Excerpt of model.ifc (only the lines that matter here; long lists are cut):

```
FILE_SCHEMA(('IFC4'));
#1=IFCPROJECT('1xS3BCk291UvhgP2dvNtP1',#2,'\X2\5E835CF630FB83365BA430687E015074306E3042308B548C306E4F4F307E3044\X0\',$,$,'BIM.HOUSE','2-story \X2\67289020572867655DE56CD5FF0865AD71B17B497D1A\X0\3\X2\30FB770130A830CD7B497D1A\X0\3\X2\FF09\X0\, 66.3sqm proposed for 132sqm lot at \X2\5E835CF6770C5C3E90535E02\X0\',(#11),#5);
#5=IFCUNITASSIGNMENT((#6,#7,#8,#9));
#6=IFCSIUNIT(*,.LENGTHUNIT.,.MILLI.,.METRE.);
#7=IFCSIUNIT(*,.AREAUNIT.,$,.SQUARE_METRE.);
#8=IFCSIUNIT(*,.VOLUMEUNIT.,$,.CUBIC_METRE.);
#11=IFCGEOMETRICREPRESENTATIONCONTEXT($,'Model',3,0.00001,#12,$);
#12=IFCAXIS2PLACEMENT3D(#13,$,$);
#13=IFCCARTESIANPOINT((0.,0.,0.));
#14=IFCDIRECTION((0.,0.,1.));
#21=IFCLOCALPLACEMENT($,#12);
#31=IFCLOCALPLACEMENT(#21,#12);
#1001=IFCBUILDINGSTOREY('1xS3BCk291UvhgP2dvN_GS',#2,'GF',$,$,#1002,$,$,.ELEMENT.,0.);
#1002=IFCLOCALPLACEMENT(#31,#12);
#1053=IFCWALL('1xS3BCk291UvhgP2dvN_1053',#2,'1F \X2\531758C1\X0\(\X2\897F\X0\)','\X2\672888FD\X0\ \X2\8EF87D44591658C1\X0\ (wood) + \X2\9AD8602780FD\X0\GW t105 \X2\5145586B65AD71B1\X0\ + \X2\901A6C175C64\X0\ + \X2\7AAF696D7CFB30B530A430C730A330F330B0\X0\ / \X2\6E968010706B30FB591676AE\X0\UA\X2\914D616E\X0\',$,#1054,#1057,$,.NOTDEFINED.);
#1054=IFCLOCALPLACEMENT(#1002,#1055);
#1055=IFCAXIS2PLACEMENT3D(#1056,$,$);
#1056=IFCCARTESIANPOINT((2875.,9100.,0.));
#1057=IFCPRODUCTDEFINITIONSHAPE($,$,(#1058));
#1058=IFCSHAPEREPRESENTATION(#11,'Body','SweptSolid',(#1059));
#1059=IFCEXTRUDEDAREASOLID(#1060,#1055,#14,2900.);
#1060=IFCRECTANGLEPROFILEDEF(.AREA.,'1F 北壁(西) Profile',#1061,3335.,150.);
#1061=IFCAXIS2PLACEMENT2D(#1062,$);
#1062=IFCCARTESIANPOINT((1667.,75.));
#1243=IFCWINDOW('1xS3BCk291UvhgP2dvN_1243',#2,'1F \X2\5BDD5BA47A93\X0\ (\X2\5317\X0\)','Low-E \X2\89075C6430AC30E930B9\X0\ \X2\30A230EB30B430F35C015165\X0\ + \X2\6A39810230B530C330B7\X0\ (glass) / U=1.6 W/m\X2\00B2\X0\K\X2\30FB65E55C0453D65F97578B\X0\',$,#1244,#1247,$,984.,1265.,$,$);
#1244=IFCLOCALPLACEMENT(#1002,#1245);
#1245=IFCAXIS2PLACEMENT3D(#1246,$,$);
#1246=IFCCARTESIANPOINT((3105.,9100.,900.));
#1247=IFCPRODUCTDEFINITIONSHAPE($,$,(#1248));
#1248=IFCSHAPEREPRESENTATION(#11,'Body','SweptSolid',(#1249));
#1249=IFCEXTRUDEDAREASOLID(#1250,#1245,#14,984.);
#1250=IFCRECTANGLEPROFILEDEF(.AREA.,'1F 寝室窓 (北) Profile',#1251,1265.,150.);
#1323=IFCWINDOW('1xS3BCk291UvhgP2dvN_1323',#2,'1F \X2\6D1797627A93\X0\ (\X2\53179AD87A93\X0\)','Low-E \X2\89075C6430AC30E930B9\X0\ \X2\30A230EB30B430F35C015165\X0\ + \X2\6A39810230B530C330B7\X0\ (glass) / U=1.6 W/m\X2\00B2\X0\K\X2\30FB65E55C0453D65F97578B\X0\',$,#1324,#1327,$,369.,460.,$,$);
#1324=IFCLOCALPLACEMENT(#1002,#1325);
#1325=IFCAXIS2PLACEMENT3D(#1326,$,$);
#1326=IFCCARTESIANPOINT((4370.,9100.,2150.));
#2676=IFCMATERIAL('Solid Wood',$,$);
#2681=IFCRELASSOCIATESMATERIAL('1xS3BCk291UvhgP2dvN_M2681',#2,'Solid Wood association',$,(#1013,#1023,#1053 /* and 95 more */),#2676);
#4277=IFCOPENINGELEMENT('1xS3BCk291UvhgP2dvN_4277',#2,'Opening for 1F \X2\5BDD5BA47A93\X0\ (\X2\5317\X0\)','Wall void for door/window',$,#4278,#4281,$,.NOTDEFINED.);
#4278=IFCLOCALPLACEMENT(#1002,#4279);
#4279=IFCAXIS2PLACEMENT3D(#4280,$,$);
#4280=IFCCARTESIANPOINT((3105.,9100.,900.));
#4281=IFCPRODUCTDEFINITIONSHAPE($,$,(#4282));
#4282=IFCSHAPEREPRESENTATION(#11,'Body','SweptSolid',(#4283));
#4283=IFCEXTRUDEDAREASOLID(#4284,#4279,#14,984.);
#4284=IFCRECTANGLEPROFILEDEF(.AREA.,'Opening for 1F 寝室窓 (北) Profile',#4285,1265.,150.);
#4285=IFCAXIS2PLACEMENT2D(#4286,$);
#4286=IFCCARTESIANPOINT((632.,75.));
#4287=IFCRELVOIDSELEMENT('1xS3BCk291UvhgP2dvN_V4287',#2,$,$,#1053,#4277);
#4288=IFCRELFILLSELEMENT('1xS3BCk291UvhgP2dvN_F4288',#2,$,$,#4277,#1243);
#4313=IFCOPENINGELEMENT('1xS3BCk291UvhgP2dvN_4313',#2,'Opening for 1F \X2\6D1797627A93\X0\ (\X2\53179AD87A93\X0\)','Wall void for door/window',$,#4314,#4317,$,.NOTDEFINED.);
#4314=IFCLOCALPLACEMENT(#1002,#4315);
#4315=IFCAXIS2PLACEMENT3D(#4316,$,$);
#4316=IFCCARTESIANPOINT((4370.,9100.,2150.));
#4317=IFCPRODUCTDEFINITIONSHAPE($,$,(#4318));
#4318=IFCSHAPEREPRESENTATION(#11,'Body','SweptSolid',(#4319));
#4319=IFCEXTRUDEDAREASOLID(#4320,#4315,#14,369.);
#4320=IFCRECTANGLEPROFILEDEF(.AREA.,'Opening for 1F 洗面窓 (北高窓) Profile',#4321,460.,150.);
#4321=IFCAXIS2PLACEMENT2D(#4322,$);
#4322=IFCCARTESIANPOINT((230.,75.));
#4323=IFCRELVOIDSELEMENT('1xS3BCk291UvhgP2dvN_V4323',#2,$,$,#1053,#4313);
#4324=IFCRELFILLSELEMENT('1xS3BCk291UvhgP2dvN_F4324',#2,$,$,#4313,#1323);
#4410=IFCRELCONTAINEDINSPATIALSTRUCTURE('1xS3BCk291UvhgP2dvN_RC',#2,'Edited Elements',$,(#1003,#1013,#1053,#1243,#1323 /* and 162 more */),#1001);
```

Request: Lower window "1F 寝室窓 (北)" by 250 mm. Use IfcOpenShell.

```python
import numpy as np
import ifcopenshell
import ifcopenshell.api.geometry
import ifcopenshell.util.placement
import ifcopenshell.util.unit

model = ifcopenshell.open("model.ifc")
unit_scale = ifcopenshell.util.unit.calculate_unit_scale(model)

window = model.by_guid("1xS3BCk291UvhgP2dvN_1243")
opening = window.FillsVoids[0].RelatingOpeningElement
dz = -250.0

shift = np.array([0.0, 0.0, dz])
# The window is not placed relative to its opening, so move both.
for product in (opening, window):
    matrix = ifcopenshell.util.placement.get_local_placement(product.ObjectPlacement)
    matrix[:3, 3] += shift
    ifcopenshell.api.geometry.edit_object_placement(model, product=product, matrix=matrix, is_si=False)

print(f"moved by {dz * unit_scale:+.3f} m")

model.write("model_rev.ifc")
```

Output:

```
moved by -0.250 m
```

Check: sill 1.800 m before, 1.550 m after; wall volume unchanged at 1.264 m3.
